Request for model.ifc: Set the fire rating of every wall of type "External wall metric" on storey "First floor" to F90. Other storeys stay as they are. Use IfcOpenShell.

First a look at what the model holds.

```python
import ifcopenshell
import ifcopenshell.util.element

model = ifcopenshell.open("model.ifc")
print(model.schema)
storey = next(s for s in model.by_type("IfcBuildingStorey") if s.Name == "First floor")
walls = [e for e in ifcopenshell.util.element.get_decomposition(storey) if e.is_a("IfcWall")]
seen = {}
for e in walls:
    element_type = ifcopenshell.util.element.get_type(e)
    key = (element_type.Name if element_type != e and element_type else None, ifcopenshell.util.element.get_pset(e, "Pset_WallCommon", "FireRating"))
    seen[key] = seen.get(key, 0) + 1
for (name, value), count in sorted(seen.items(), key=str):
    print(count, "x", name, "|", value)
```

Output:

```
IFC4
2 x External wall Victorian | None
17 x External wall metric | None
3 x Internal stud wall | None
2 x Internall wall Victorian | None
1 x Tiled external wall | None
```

```python
import ifcopenshell
import ifcopenshell.api.pset
import ifcopenshell.util.element

model = ifcopenshell.open("model.ifc")

storey = next(s for s in model.by_type("IfcBuildingStorey") if s.Name == "First floor")
walls = [e for e in ifcopenshell.util.element.get_decomposition(storey) if e.is_a("IfcWall")]

count = 0
for e in walls:
    element_type = ifcopenshell.util.element.get_type(e)
    if element_type in (None, e) or element_type.Name != "External wall metric":
        continue
    # add_pset returns the element's existing set when there is one.
    pset = ifcopenshell.api.pset.add_pset(model, product=e, name="Pset_WallCommon")
    ifcopenshell.api.pset.edit_pset(model, pset=pset, properties={"FireRating": "F90"})
    count += 1

print(count, "walls updated")

model.write("model_updated.ifc")
```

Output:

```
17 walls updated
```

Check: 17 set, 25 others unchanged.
